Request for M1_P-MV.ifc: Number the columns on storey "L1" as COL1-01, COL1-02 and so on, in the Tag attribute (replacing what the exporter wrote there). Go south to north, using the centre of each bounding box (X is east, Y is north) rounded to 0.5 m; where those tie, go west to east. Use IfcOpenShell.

First a look at what the model holds.

```python
import ifcopenshell
import ifcopenshell.util.element
import ifcopenshell.util.placement

model = ifcopenshell.open("M1_P-MV.ifc")
print(model.schema)
storey = next(s for s in model.by_type("IfcBuildingStorey") if s.Name == "L1")
columns = [e for e in ifcopenshell.util.element.get_decomposition(storey) if e.is_a("IfcColumn")]
for e in sorted(columns, key=lambda e: e.id()):
    origin = ifcopenshell.util.placement.get_local_placement(e.ObjectPlacement)[:3, 3]
    print(e.id(), e.Tag, e.Name, origin.round(2) + 0.0, sep=" | ")
```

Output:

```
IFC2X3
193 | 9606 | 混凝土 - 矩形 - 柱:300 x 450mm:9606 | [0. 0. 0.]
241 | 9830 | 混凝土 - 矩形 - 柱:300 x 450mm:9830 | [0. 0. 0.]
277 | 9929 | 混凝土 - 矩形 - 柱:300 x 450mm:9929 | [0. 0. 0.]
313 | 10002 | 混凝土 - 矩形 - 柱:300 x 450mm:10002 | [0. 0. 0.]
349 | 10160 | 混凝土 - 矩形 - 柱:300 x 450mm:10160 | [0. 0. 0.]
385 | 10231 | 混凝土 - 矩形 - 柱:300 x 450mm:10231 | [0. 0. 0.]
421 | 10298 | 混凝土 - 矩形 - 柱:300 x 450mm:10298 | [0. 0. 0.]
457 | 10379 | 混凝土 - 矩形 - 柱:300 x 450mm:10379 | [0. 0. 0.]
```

```python
import ifcopenshell
import ifcopenshell.geom
import ifcopenshell.util.element
import ifcopenshell.util.shape

model = ifcopenshell.open("M1_P-MV.ifc")
settings = ifcopenshell.geom.settings()
settings.set("use-world-coords", True)


def centre(element):
    shape = ifcopenshell.geom.create_shape(settings, element)
    return ifcopenshell.util.shape.get_bbox_centroid(shape.geometry)


storey = next(s for s in model.by_type("IfcBuildingStorey") if s.Name == "L1")
columns = [e for e in ifcopenshell.util.element.get_decomposition(storey) if e.is_a("IfcColumn")]

# Insertion points can sit at a corner or the storey origin, so sort by the geometry (in metres).
centres = {e: centre(e) for e in columns}
columns.sort(key=lambda e: (round(centres[e][1] / 0.5), centres[e][0]))

for i, e in enumerate(columns, start=1):
    number = f"COL1-{i:02d}"
    e.Tag = number
    print(e.id(), number)

model.write("M1_P-MV_updated.ifc")
```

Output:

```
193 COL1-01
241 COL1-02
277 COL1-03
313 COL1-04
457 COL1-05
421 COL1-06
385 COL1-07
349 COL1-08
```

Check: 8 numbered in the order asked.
